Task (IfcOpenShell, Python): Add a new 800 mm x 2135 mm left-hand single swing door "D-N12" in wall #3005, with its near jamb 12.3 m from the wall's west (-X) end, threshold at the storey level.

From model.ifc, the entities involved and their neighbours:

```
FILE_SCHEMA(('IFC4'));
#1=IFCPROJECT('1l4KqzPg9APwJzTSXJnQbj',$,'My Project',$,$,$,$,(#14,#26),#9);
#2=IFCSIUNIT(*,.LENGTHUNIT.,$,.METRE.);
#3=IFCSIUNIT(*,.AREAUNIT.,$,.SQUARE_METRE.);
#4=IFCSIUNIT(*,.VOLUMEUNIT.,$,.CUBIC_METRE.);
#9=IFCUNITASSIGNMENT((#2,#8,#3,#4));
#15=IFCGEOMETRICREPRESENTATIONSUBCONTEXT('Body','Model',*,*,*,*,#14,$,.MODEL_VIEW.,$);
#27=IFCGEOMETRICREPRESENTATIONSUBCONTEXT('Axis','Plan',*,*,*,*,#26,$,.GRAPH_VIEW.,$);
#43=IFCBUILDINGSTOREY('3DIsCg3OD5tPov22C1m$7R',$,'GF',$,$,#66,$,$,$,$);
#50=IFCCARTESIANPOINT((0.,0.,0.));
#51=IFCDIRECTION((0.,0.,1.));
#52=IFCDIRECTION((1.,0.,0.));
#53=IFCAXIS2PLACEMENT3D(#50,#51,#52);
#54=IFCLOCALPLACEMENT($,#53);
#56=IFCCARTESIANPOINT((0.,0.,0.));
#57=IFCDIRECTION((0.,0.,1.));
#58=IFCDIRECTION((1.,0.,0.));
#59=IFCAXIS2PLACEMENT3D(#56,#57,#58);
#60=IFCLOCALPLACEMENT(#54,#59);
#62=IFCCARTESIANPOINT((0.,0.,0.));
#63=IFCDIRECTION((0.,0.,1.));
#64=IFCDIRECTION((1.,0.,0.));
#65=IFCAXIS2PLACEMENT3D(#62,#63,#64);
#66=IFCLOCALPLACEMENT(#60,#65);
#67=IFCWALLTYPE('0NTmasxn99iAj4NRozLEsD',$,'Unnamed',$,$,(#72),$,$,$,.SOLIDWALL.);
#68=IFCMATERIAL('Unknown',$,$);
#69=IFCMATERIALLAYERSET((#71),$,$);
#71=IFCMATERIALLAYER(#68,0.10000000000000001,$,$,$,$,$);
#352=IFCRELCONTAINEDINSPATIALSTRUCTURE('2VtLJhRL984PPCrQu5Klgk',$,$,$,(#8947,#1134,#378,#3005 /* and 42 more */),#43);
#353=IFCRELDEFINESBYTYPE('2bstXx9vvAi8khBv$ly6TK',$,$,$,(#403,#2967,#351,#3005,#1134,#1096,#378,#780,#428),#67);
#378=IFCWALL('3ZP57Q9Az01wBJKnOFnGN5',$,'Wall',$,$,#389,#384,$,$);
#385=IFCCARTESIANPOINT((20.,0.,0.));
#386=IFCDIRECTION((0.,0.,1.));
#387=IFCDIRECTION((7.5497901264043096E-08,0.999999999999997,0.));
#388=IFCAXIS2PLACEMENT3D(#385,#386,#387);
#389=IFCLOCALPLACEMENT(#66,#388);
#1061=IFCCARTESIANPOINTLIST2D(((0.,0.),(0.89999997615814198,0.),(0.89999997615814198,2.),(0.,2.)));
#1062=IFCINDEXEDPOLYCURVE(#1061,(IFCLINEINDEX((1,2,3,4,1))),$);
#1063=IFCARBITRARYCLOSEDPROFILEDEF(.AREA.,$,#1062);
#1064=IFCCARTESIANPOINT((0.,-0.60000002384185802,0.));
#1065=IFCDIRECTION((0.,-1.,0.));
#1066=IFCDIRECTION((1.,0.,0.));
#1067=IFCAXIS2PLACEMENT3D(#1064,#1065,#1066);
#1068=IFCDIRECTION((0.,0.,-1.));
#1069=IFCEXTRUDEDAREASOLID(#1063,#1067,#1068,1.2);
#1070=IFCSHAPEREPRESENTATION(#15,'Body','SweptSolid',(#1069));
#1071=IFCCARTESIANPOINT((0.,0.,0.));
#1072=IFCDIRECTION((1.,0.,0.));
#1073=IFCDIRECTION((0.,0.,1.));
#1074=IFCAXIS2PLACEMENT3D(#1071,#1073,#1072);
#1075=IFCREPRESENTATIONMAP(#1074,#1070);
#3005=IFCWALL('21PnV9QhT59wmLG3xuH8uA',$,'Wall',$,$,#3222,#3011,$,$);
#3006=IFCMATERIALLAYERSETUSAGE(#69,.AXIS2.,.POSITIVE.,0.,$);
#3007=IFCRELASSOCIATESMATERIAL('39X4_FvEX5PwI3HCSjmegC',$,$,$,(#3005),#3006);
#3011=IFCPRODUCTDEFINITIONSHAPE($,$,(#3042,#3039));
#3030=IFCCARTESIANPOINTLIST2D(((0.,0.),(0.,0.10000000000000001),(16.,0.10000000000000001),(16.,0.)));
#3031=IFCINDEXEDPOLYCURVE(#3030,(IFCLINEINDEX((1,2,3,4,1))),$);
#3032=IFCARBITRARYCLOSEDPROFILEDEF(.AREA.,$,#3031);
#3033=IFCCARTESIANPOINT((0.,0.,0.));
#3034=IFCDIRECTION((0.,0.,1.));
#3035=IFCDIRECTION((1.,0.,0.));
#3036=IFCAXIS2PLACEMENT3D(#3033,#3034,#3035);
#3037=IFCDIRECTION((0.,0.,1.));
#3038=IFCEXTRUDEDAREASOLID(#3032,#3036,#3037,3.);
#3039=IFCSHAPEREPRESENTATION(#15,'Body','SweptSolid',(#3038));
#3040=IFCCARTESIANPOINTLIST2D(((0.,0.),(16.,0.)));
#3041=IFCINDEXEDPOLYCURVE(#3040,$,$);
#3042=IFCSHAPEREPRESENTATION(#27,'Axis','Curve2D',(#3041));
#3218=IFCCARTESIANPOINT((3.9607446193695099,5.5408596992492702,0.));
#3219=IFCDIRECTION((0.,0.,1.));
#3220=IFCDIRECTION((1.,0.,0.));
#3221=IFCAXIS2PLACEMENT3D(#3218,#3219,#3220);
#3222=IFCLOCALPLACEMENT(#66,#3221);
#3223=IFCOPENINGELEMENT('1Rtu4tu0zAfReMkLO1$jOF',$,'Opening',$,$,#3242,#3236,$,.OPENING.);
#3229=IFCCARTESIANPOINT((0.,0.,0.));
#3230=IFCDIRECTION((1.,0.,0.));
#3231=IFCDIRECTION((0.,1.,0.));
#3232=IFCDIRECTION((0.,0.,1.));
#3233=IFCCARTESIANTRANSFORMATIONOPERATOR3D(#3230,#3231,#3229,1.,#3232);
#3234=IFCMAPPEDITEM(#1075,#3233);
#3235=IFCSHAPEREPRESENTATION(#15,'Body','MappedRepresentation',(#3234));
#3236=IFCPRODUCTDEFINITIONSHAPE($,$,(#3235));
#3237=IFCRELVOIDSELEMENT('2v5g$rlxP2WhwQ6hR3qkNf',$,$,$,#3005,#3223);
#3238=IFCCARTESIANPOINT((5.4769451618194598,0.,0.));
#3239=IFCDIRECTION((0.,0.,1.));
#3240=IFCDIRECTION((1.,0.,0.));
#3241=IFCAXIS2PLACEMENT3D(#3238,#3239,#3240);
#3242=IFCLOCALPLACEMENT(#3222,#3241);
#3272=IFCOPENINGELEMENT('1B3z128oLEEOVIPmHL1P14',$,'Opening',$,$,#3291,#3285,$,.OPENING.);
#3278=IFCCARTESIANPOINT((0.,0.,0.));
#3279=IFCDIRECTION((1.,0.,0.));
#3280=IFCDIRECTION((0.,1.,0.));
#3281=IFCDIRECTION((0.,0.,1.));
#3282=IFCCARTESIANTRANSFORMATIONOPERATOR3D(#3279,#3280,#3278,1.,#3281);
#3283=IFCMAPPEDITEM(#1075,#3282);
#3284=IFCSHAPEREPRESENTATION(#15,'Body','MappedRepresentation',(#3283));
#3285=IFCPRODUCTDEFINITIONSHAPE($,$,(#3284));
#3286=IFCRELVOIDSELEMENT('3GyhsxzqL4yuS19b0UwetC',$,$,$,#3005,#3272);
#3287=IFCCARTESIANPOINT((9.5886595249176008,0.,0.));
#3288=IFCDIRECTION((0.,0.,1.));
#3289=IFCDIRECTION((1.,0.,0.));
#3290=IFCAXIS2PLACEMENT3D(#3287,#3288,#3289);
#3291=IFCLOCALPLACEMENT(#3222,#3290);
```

```python
import numpy as np
import ifcopenshell
import ifcopenshell.api.feature
import ifcopenshell.api.geometry
import ifcopenshell.api.root
import ifcopenshell.api.spatial
import ifcopenshell.geom
import ifcopenshell.util.element
import ifcopenshell.util.placement
import ifcopenshell.util.representation
import ifcopenshell.util.shape
import ifcopenshell.util.unit

model = ifcopenshell.open("model.ifc")
unit_scale = ifcopenshell.util.unit.calculate_unit_scale(model)
settings = ifcopenshell.geom.settings()


def volume(element):
    """Net volume in cubic metres, openings subtracted."""
    shape = ifcopenshell.geom.create_shape(settings, element)
    return ifcopenshell.util.shape.get_volume(shape.geometry)


wall = model.by_guid("21PnV9QhT59wmLG3xuH8uA")
storey = ifcopenshell.util.element.get_container(wall, ifc_class="IfcBuildingStorey")
context = ifcopenshell.util.representation.get_context(model, "Model", "Body", "MODEL_VIEW")
before = volume(wall)

width, height, from_end, sill = 0.8, 2.135, 12.3, 0.0  # metres

# The wall runs along its own X axis, and the end named is its -X end.
wall_shape = ifcopenshell.geom.create_shape(settings, wall)
x, y, z = ifcopenshell.util.shape.get_vertices(wall_shape.geometry).T
start = x.min() + from_end
face, thickness = float(y.min()), float(y.max() - y.min())
wall_matrix = ifcopenshell.util.placement.get_local_placement(wall.ObjectPlacement)
level = ifcopenshell.util.placement.get_local_placement(storey.ObjectPlacement)[2, 3]


def in_wall(x, y):
    """Placement at x, y metres in the wall's axes, at sill height."""
    matrix = wall_matrix.copy()
    matrix[:, 3] = wall_matrix @ np.array([x / unit_scale, y / unit_scale, 0.0, 1.0])
    matrix[2, 3] = level + sill / unit_scale
    return matrix


# Opening: a box that overshoots both wall faces by 50 mm.
opening = ifcopenshell.api.root.create_entity(model, ifc_class="IfcOpeningElement", predefined_type="OPENING")
box = ifcopenshell.api.geometry.add_wall_representation(
    model, context=context, length=width, height=height, thickness=thickness + 0.1
)
ifcopenshell.api.geometry.assign_representation(model, product=opening, representation=box)
ifcopenshell.api.geometry.edit_object_placement(model, product=opening, matrix=in_wall(start, face - 0.05), is_si=False)
ifcopenshell.api.feature.add_feature(model, feature=opening, element=wall)

door = ifcopenshell.api.root.create_entity(model, ifc_class="IfcDoor", name="D-N12", predefined_type="DOOR")
door.OverallWidth, door.OverallHeight = width / unit_scale, height / unit_scale
door.OperationType = "SINGLE_SWING_LEFT"
body = ifcopenshell.api.geometry.add_door_representation(
    model,
    context=context,
    overall_width=door.OverallWidth,
    overall_height=door.OverallHeight,
    operation_type="SINGLE_SWING_LEFT",
    lining_properties={"LiningDepth": thickness / unit_scale, "ThresholdDepth": thickness / unit_scale},
)
ifcopenshell.api.geometry.assign_representation(model, product=door, representation=body)
ifcopenshell.api.spatial.assign_container(model, products=[door], relating_structure=storey)
ifcopenshell.api.feature.add_filling(model, opening=opening, element=door)

# The lining spans the wall, so the door starts at the wall face.
ifcopenshell.api.geometry.edit_object_placement(model, product=door, matrix=in_wall(start, face), is_si=False)

after = volume(wall)

print(f"wall volume {before:.3f} -> {after:.3f} m3")

model.write("model-out.ifc")
```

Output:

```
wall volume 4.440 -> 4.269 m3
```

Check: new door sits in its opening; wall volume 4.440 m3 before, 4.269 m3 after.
